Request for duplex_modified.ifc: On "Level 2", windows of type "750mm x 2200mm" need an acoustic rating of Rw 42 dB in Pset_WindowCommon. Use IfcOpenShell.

First a look at what the model holds.

```python
import ifcopenshell
import ifcopenshell.util.element

model = ifcopenshell.open("duplex_modified.ifc")
print(model.schema)
storey = next(s for s in model.by_type("IfcBuildingStorey") if s.Name == "Level 2")
windows = [e for e in ifcopenshell.util.element.get_decomposition(storey) if e.is_a("IfcWindow")]
seen = {}
for e in windows:
    element_type = ifcopenshell.util.element.get_type(e)
    key = (element_type.Name if element_type != e and element_type else None, ifcopenshell.util.element.get_pset(e, "Pset_WindowCommon", "AcousticRating"))
    seen[key] = seen.get(key, 0) + 1
for (name, value), count in sorted(seen.items(), key=str):
    print(count, "x", name, "|", value)
```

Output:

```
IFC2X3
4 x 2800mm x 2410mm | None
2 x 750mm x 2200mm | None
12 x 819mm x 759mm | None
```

```python
import ifcopenshell
import ifcopenshell.api.pset
import ifcopenshell.util.element

model = ifcopenshell.open("duplex_modified.ifc")

storey = next(s for s in model.by_type("IfcBuildingStorey") if s.Name == "Level 2")
windows = [e for e in ifcopenshell.util.element.get_decomposition(storey) if e.is_a("IfcWindow")]

count = 0
for e in windows:
    element_type = ifcopenshell.util.element.get_type(e)
    if element_type in (None, e) or element_type.Name != "750mm x 2200mm":
        continue
    # add_pset returns the element's existing set when there is one.
    pset = ifcopenshell.api.pset.add_pset(model, product=e, name="Pset_WindowCommon")
    ifcopenshell.api.pset.edit_pset(model, pset=pset, properties={"AcousticRating": "Rw 42 dB"})
    count += 1

print(count, "windows updated")

model.write("duplex_modified_updated.ifc")
```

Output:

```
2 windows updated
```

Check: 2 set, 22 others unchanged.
